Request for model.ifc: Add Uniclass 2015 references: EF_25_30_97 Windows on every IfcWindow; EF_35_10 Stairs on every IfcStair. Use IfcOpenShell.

First a look at what the model holds.

```python
import ifcopenshell

model = ifcopenshell.open("model.ifc")
print(model.schema)
print("classifications:", [c.Name for c in model.by_type("IfcClassification")])
for ifc_class in ("IfcDoor", "IfcRoof", "IfcStair", "IfcWall", "IfcWindow"):
    print(ifc_class, len(model.by_type(ifc_class)))
```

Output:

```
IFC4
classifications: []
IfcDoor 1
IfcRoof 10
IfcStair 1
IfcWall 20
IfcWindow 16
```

```python
import ifcopenshell
import ifcopenshell.api.classification

model = ifcopenshell.open("model.ifc")

system = ifcopenshell.api.classification.add_classification(model, classification="Uniclass 2015")

codes = {
    "IfcWindow": ("EF_25_30_97", "Windows"),
    "IfcStair": ("EF_35_10", "Stairs"),
}
for ifc_class, (code, name) in codes.items():
    products = model.by_type(ifc_class)
    ifcopenshell.api.classification.add_reference(
        model, products=products, classification=system, identification=code, name=name
    )
    print(code, len(products))

model.write("model_updated.ifc")
```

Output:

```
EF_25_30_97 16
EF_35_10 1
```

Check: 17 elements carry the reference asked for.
